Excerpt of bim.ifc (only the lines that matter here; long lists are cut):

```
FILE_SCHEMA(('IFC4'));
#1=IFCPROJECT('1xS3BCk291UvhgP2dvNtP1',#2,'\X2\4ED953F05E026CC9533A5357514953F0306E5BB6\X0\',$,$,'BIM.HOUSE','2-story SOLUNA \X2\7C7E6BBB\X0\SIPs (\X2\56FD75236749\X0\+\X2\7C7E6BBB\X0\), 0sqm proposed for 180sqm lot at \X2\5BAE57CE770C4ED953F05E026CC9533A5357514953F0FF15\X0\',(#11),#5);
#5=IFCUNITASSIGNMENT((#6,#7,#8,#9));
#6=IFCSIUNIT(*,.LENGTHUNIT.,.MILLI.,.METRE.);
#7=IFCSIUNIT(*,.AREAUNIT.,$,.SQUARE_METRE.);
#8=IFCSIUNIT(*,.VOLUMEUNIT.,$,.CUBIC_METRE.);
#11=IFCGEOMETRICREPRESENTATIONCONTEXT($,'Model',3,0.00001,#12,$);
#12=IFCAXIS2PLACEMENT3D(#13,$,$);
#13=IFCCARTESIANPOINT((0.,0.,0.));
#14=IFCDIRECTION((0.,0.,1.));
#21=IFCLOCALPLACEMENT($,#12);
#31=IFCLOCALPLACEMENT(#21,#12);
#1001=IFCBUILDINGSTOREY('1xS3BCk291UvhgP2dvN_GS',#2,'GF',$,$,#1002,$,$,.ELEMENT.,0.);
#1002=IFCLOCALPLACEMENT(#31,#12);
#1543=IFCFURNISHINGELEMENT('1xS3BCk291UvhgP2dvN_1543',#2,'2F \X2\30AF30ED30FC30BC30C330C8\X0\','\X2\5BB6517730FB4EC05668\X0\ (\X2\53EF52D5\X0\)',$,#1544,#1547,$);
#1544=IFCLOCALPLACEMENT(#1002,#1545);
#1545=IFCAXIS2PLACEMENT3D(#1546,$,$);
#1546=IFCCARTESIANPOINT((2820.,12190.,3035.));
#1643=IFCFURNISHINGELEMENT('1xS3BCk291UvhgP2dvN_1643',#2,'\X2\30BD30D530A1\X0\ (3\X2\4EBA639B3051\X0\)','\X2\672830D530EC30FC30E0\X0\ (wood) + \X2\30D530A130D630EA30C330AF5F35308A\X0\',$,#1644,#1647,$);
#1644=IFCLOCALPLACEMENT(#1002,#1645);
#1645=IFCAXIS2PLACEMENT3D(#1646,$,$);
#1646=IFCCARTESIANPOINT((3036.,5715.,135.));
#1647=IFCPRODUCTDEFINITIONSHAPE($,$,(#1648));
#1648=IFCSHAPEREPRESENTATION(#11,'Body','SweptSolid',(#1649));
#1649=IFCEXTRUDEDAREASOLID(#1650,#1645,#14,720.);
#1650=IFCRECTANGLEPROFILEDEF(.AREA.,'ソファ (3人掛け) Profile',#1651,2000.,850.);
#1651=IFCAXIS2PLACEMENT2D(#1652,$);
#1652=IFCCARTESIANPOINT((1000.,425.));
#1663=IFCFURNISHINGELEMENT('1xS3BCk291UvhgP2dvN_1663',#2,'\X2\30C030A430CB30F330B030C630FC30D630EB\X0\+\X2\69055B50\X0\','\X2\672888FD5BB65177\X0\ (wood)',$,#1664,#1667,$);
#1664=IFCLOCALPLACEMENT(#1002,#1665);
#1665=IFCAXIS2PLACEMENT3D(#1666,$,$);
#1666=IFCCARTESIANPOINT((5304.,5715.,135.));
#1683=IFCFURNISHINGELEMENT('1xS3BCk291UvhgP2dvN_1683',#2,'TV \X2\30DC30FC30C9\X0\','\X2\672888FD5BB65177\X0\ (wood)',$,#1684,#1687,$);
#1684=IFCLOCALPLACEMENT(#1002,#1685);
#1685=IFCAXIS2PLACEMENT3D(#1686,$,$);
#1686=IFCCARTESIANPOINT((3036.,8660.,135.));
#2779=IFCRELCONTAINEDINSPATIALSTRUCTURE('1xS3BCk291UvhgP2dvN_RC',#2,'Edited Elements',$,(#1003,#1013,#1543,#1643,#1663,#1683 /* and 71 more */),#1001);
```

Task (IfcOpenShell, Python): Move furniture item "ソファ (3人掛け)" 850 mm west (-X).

```python
import ifcopenshell
import ifcopenshell.api.geometry
import ifcopenshell.util.placement
import ifcopenshell.util.unit

model = ifcopenshell.open("bim.ifc")
unit_scale = ifcopenshell.util.unit.calculate_unit_scale(model)

item = model.by_id(1643)
matrix = ifcopenshell.util.placement.get_local_placement(item.ObjectPlacement)
matrix[0, 3] -= 0.85 / unit_scale
ifcopenshell.api.geometry.edit_object_placement(model, product=item, matrix=matrix, is_si=False)

print(ifcopenshell.util.placement.get_local_placement(item.ObjectPlacement).round(3) + 0.0)

model.write("bim_edited.ifc")
```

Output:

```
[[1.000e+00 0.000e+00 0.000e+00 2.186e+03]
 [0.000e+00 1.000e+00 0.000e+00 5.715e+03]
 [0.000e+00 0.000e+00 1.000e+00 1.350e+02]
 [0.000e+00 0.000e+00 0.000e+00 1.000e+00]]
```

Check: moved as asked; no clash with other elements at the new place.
